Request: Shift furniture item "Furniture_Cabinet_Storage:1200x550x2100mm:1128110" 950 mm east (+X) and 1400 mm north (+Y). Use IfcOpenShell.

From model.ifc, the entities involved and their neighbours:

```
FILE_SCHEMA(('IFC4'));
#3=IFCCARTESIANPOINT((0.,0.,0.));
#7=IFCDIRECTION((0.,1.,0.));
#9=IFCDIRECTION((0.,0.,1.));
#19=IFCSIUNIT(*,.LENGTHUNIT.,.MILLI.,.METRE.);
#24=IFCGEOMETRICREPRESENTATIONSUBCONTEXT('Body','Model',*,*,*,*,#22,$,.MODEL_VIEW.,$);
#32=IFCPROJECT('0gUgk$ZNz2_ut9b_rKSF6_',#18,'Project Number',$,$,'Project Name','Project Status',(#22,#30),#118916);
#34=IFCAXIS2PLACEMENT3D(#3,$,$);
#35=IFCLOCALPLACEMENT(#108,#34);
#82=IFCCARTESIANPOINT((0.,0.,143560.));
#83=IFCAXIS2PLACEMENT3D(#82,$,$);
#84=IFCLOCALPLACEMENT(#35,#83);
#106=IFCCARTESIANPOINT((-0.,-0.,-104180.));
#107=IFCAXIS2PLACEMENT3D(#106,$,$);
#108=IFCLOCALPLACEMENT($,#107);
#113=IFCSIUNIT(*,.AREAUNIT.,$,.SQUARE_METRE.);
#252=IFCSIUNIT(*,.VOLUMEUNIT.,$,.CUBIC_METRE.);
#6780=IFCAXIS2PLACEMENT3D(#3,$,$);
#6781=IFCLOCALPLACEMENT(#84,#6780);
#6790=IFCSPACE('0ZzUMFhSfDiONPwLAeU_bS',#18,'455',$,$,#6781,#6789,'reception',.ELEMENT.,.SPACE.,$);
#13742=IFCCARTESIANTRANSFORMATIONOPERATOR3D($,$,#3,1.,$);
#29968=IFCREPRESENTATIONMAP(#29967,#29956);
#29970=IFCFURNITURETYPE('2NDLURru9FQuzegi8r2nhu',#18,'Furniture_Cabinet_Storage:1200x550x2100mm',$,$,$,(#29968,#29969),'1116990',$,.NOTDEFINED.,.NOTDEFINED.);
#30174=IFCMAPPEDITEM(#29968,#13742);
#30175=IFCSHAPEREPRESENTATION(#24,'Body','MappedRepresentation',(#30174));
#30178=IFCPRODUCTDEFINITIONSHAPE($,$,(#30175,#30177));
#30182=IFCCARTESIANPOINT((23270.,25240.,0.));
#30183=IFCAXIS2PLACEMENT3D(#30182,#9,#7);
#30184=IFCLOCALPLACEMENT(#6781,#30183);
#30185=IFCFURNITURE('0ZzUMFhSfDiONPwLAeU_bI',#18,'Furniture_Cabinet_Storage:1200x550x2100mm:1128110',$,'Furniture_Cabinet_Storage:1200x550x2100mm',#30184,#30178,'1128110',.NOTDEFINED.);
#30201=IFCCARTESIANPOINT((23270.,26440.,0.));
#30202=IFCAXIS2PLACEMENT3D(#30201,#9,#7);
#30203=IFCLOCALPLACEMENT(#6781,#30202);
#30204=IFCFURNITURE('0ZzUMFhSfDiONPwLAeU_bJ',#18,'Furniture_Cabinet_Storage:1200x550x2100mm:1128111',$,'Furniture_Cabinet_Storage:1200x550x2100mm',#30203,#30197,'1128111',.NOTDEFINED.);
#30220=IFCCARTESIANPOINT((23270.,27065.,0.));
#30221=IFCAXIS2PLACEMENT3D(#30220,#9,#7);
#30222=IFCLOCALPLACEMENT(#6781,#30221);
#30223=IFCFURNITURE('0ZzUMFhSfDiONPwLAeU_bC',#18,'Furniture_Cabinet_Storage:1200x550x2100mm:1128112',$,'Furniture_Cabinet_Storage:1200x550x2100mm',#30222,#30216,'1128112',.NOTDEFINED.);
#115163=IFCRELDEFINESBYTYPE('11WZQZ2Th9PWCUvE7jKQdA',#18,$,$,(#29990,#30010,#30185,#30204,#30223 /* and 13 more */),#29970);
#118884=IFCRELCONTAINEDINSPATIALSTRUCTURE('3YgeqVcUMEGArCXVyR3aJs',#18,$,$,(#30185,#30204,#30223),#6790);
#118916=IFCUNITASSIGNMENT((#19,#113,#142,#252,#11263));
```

```python
import ifcopenshell
import ifcopenshell.api.geometry
import ifcopenshell.util.placement

model = ifcopenshell.open("model.ifc")

item = model.by_guid("0ZzUMFhSfDiONPwLAeU_bI")
matrix = ifcopenshell.util.placement.get_local_placement(item.ObjectPlacement)
matrix[0, 3] += 950.0
matrix[1, 3] += 1400.0
ifcopenshell.api.geometry.edit_object_placement(model, product=item, matrix=matrix, is_si=False)

print(ifcopenshell.util.placement.get_local_placement(item.ObjectPlacement).round(3) + 0.0)

model.write("model_edited.ifc")
```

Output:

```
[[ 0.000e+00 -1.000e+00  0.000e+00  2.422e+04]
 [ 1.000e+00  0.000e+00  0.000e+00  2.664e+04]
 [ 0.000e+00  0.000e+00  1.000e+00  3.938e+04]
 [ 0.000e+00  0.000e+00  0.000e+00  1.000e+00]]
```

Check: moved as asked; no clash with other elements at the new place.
